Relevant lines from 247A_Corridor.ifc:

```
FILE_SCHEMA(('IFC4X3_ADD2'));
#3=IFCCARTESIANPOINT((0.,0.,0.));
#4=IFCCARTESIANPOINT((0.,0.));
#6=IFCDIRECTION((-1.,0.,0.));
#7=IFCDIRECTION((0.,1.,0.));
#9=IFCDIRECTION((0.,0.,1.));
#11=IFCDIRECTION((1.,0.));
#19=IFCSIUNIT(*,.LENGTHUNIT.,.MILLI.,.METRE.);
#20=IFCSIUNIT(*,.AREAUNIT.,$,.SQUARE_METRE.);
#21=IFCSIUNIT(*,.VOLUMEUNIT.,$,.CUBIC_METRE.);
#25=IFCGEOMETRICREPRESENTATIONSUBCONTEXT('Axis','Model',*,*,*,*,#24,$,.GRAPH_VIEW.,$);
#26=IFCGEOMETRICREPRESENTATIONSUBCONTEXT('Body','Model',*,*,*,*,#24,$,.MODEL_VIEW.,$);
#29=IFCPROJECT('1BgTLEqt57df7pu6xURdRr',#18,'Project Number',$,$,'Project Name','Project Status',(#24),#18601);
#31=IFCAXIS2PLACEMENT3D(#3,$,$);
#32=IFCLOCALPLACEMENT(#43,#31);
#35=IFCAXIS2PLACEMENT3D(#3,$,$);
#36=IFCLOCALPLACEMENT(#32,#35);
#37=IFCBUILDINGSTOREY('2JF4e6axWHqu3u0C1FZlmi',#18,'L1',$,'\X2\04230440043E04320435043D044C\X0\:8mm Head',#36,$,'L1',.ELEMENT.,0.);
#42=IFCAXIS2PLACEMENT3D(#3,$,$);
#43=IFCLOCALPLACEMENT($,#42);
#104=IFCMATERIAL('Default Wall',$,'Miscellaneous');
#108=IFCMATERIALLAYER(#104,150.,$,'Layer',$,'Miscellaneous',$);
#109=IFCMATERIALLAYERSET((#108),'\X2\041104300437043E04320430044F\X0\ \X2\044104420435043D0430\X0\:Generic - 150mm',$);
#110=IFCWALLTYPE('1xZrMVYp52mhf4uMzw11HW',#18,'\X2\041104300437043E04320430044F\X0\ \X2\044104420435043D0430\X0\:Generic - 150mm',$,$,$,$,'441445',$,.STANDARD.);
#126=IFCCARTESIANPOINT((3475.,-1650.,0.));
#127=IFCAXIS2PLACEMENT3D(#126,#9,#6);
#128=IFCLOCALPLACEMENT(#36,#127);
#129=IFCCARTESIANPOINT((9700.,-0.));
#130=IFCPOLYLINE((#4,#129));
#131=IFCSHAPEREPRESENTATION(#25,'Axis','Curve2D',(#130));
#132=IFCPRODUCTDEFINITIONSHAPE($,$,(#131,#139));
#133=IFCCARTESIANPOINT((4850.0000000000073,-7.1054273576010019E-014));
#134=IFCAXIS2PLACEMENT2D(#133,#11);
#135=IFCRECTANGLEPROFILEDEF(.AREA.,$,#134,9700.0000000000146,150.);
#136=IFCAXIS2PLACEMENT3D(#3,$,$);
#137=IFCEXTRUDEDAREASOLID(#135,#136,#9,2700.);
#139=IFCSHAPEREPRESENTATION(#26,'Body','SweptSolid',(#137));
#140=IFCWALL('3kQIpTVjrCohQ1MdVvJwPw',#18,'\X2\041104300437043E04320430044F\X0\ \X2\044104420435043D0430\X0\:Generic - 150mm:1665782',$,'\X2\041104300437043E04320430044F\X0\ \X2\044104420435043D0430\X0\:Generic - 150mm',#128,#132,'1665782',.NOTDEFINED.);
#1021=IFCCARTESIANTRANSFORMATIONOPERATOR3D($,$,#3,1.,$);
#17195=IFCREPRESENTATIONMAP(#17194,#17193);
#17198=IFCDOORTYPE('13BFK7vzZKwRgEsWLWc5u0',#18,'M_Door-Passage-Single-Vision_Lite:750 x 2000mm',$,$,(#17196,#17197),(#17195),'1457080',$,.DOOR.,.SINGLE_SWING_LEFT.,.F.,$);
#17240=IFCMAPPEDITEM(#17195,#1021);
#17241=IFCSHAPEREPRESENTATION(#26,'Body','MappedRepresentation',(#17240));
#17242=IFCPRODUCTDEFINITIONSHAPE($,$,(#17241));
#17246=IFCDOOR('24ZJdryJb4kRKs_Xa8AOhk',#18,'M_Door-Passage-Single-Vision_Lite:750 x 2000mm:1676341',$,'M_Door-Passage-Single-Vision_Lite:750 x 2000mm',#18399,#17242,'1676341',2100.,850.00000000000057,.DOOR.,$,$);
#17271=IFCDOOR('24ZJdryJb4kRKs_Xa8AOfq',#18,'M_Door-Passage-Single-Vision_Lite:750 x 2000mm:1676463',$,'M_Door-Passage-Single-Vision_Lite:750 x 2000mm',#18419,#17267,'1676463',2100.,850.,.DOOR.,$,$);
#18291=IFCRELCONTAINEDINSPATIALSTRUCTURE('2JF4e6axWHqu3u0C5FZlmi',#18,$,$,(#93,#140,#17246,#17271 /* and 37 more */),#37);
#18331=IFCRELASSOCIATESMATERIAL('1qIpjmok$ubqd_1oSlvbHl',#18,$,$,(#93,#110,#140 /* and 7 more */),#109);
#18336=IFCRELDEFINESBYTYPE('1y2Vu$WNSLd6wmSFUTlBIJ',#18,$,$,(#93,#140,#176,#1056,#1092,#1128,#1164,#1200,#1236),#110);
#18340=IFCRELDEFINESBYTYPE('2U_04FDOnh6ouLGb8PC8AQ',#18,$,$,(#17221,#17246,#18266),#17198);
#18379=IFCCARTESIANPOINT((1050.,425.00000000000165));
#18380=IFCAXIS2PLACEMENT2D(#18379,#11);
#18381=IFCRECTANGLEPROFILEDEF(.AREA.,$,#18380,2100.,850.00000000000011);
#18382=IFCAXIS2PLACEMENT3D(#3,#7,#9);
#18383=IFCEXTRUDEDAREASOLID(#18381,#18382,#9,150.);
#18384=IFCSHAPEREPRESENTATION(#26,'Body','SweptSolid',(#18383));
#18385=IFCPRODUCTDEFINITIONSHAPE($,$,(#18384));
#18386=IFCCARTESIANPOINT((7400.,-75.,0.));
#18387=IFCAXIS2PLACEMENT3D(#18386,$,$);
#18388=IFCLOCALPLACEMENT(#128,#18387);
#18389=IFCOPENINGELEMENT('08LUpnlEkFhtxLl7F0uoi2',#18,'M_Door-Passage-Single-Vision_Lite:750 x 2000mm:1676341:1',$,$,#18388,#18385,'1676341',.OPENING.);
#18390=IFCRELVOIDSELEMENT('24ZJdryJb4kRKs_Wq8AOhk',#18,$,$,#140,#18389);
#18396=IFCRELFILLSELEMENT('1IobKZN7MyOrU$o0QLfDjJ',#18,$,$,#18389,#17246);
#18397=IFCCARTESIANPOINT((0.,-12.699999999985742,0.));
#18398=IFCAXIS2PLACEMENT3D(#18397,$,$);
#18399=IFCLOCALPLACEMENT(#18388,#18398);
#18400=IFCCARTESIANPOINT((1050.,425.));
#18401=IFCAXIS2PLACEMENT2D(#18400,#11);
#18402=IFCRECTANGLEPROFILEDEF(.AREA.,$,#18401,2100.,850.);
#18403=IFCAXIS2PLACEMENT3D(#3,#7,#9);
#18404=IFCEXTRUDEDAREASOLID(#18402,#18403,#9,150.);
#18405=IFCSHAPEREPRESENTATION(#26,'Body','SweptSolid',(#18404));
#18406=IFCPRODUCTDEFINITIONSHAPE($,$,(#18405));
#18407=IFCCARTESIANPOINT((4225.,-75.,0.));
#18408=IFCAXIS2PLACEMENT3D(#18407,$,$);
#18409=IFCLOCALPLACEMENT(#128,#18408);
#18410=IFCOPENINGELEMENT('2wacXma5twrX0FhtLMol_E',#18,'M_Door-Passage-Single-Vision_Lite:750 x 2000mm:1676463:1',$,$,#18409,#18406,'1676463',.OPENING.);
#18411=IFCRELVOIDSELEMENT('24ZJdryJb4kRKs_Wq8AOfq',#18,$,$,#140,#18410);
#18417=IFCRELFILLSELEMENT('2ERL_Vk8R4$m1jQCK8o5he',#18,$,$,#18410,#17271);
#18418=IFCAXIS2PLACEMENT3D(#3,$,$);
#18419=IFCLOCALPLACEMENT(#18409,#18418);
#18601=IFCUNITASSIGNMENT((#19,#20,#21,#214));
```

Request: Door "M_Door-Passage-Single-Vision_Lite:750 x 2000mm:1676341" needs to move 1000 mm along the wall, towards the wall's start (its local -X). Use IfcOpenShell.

```python
import ifcopenshell
import ifcopenshell.api.geometry
import ifcopenshell.util.placement

model = ifcopenshell.open("247A_Corridor.ifc")

door = model.by_id(17246)
opening = door.FillsVoids[0].RelatingOpeningElement
wall = opening.VoidsElements[0].RelatingBuildingElement

wall_matrix = ifcopenshell.util.placement.get_local_placement(wall.ObjectPlacement)
shift = wall_matrix[:3, 0] * -1000.0
before = ifcopenshell.util.placement.get_local_placement(door.ObjectPlacement)[:3, 3].copy()

# The door is placed relative to its opening, so it follows when the opening moves.
matrix = ifcopenshell.util.placement.get_local_placement(opening.ObjectPlacement)
matrix[:3, 3] += shift
ifcopenshell.api.geometry.edit_object_placement(
    model, product=opening, matrix=matrix, is_si=False, should_transform_children=True
)

after = ifcopenshell.util.placement.get_local_placement(door.ObjectPlacement)[:3, 3]
print("door moved by", (after - before).round(3) + 0.0)

model.write("247A_Corridor-out.ifc")
```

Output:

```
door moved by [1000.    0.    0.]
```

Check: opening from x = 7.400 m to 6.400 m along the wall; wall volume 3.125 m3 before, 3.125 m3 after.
